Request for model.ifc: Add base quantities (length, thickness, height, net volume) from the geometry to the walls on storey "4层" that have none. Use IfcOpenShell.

First a look at what the model holds.

```python
import ifcopenshell
import ifcopenshell.util.element
import ifcopenshell.util.unit

model = ifcopenshell.open("model.ifc")
print(model.schema)
for unit_type in ("LENGTHUNIT", "AREAUNIT", "VOLUMEUNIT"):
    print(unit_type, ifcopenshell.util.unit.calculate_unit_scale(model, unit_type))
storey = next(s for s in model.by_type("IfcBuildingStorey") if s.Name == "4层")
walls = [e for e in ifcopenshell.util.element.get_decomposition(storey) if e.is_a("IfcWall")]
for e in sorted(walls, key=lambda e: e.id()):
    print(e.id(), e.is_a(), e.Name, list(ifcopenshell.util.element.get_psets(e, qtos_only=True)), sep=" | ")
```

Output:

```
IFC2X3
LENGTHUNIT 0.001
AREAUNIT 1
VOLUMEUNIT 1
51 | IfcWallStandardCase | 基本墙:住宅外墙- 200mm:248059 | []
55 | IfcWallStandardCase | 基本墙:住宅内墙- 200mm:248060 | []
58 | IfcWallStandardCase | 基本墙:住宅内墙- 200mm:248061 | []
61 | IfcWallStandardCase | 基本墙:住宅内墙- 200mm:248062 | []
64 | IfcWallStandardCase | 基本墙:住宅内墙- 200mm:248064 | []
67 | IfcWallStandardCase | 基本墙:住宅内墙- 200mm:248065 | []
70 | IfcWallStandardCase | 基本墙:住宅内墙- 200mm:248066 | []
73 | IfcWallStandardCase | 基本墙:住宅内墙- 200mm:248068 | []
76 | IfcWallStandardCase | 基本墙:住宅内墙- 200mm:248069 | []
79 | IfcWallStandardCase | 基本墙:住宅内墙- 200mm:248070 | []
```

```python
import ifcopenshell
import ifcopenshell.api.pset
import ifcopenshell.geom
import ifcopenshell.util.element
import ifcopenshell.util.shape
import ifcopenshell.util.unit

model = ifcopenshell.open("model.ifc")
unit_scale = ifcopenshell.util.unit.calculate_unit_scale(model)
volume_scale = ifcopenshell.util.unit.calculate_unit_scale(model, "VOLUMEUNIT")
settings = ifcopenshell.geom.settings()

storey = next(s for s in model.by_type("IfcBuildingStorey") if s.Name == "4层")
walls = [e for e in ifcopenshell.util.element.get_decomposition(storey) if e.is_a("IfcWall")]

for e in sorted(walls, key=lambda e: e.id()):
    if ifcopenshell.util.element.get_psets(e, qtos_only=True, should_inherit=False):
        continue
    # Geometry comes back in metres, in the element's own axes.
    shape = ifcopenshell.geom.create_shape(settings, e)
    values = {
        "Length": ifcopenshell.util.shape.get_x(shape.geometry) / unit_scale,
        "Width": ifcopenshell.util.shape.get_y(shape.geometry) / unit_scale,
        "Height": ifcopenshell.util.shape.get_z(shape.geometry) / unit_scale,
        "NetVolume": ifcopenshell.util.shape.get_volume(shape.geometry) / volume_scale,
    }
    qto = ifcopenshell.api.pset.add_qto(model, product=e, name="BaseQuantities")
    ifcopenshell.api.pset.edit_qto(model, qto=qto, properties=values)
    print(e.id(), {k: round(v, 3) for k, v in values.items()})

model.write("model_v2.ifc")
```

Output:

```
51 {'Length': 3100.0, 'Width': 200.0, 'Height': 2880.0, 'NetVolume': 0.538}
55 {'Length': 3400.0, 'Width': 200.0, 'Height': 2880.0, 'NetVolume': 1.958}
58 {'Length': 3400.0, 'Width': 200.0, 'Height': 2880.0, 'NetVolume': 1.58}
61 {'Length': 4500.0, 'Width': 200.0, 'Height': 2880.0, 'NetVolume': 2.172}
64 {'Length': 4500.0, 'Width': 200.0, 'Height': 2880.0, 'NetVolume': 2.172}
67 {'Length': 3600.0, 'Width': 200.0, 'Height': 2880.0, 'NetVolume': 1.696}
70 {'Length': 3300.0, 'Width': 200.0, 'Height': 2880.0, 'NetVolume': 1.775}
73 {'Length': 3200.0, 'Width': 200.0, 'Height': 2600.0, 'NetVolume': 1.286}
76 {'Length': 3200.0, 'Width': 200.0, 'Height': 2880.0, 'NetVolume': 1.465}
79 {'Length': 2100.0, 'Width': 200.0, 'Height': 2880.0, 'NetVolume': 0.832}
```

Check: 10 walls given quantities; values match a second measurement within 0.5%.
